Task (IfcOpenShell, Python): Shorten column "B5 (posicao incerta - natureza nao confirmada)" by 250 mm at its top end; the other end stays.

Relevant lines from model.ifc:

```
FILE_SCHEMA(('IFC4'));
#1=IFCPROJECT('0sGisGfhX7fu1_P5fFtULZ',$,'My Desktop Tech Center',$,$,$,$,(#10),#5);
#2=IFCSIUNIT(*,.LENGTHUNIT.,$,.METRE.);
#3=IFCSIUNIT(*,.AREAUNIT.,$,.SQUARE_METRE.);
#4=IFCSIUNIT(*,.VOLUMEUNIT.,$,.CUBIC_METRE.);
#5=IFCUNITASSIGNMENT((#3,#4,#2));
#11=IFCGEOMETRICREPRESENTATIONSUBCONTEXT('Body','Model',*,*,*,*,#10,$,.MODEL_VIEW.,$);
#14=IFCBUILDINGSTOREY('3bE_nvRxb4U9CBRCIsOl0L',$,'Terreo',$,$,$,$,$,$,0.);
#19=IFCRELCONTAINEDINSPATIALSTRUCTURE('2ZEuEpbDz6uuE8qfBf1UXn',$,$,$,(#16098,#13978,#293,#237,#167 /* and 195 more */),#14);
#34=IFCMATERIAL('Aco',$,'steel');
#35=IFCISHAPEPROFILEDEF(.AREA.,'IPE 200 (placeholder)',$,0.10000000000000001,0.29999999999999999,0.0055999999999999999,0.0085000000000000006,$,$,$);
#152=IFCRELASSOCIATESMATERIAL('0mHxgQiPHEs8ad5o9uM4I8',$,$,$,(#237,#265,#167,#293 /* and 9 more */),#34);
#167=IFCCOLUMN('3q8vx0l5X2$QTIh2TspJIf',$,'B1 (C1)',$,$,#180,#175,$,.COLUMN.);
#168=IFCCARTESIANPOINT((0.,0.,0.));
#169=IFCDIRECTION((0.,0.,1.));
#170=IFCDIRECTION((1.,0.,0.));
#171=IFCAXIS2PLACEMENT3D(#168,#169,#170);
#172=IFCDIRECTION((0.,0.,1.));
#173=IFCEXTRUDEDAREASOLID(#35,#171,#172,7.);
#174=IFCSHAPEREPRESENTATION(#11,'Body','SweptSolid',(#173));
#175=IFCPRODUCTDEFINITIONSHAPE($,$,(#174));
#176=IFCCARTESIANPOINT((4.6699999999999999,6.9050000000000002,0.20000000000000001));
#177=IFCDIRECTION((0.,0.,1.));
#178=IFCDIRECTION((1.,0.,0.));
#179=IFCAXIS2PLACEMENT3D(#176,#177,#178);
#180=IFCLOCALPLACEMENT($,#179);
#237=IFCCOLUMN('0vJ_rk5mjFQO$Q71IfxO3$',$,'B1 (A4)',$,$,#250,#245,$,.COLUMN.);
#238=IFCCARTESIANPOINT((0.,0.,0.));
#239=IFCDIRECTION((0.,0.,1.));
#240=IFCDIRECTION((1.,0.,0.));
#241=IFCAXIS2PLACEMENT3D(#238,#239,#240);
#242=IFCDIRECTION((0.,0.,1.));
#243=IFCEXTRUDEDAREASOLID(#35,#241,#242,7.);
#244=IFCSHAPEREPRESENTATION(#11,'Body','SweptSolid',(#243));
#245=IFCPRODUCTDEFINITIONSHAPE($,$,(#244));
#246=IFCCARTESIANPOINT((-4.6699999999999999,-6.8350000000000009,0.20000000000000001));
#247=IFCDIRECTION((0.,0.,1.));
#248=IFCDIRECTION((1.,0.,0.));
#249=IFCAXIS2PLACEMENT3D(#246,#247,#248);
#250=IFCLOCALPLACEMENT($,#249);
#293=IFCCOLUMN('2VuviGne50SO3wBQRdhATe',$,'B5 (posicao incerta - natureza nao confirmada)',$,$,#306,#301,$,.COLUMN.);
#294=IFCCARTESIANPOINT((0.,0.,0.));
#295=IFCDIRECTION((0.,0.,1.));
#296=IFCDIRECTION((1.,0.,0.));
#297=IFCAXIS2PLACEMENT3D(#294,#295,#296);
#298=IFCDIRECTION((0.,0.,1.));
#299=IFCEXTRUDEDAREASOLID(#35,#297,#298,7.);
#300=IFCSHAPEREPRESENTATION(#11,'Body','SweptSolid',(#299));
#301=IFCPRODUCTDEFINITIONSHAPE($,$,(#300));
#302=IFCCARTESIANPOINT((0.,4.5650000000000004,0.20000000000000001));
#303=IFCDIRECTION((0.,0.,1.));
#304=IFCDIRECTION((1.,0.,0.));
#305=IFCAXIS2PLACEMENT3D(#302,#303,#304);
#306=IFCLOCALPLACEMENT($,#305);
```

```python
import ifcopenshell
import ifcopenshell.util.representation

model = ifcopenshell.open("model.ifc")

member = model.by_id(293)
change = -0.25

# The extrusion runs towards the end named, so only its depth changes.
body = ifcopenshell.util.representation.get_representation(member, "Model", "Body")
solid = body.Items[0]
old_length = solid.Depth
solid.Depth += change

print(f"length {old_length:g} -> {solid.Depth:g}")

model.write("model_v2.ifc")
```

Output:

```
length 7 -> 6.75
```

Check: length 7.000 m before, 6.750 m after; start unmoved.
